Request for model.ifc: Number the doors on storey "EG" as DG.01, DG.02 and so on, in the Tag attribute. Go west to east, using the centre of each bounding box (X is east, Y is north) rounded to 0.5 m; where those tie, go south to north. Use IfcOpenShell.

First a look at what the model holds.

```python
import ifcopenshell
import ifcopenshell.util.element
import ifcopenshell.util.placement

model = ifcopenshell.open("model.ifc")
print(model.schema)
storey = next(s for s in model.by_type("IfcBuildingStorey") if s.Name == "EG")
doors = [e for e in ifcopenshell.util.element.get_decomposition(storey) if e.is_a("IfcDoor")]
for e in sorted(doors, key=lambda e: e.id()):
    origin = ifcopenshell.util.placement.get_local_placement(e.ObjectPlacement)[:3, 3]
    print(e.id(), e.Tag, e.Name, origin.round(2) + 0.0, sep=" | ")
```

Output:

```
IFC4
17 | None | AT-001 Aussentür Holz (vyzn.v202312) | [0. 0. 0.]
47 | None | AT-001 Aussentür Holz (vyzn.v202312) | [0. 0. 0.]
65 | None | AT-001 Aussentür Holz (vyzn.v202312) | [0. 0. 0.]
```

```python
import ifcopenshell
import ifcopenshell.geom
import ifcopenshell.util.element
import ifcopenshell.util.shape

model = ifcopenshell.open("model.ifc")
settings = ifcopenshell.geom.settings()
settings.set("use-world-coords", True)


def centre(element):
    shape = ifcopenshell.geom.create_shape(settings, element)
    return ifcopenshell.util.shape.get_bbox_centroid(shape.geometry)


storey = next(s for s in model.by_type("IfcBuildingStorey") if s.Name == "EG")
doors = [e for e in ifcopenshell.util.element.get_decomposition(storey) if e.is_a("IfcDoor")]

# Insertion points can sit at a corner or the storey origin, so sort by the geometry (in metres).
centres = {e: centre(e) for e in doors}
doors.sort(key=lambda e: (round(centres[e][0] / 0.5), centres[e][1]))

for i, e in enumerate(doors, start=1):
    number = f"DG.{i:02d}"
    e.Tag = number
    print(e.id(), number)

model.write("model_edited.ifc")
```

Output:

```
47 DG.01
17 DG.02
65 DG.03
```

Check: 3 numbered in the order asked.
